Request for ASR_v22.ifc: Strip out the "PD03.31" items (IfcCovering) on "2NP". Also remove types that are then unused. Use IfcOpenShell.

First a look at what the model holds.

```python
import ifcopenshell
import ifcopenshell.util.element

model = ifcopenshell.open("ASR_v22.ifc")
print(model.schema)
storey = next(s for s in model.by_type("IfcBuildingStorey") if s.Name == "2NP")
coverings = [e for e in ifcopenshell.util.element.get_decomposition(storey) if e.is_a("IfcCovering")]
seen = {}
for e in coverings:
    element_type = ifcopenshell.util.element.get_type(e)
    name = element_type.Name if element_type not in (None, e) else None
    seen[name] = seen.get(name, 0) + 1
for name, count in sorted(seen.items(), key=str):
    print(count, "x", name)
```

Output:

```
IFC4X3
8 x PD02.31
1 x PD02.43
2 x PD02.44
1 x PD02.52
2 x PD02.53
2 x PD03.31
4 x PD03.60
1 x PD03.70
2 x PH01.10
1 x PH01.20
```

```python
import ifcopenshell
import ifcopenshell.api.root
import ifcopenshell.util.element

model = ifcopenshell.open("ASR_v22.ifc")

storey = next(s for s in model.by_type("IfcBuildingStorey") if s.Name == "2NP")
coverings = [e for e in ifcopenshell.util.element.get_decomposition(storey) if e.is_a("IfcCovering")]
targets = [e for e in coverings if (t := ifcopenshell.util.element.get_type(e)) not in (None, e) and t.Name == "PD03.31"]
types = {ifcopenshell.util.element.get_type(e) for e in targets} - {None, *targets}

for e in targets:
    ifcopenshell.api.root.remove_product(model, product=e)
print(len(targets), "removed")

unused = [t for t in types if not ifcopenshell.util.element.get_types(t)]
for t in unused:
    ifcopenshell.api.root.remove_product(model, product=t)
print(len(unused), "unused types removed")

model.write("ASR_v22_updated.ifc")
```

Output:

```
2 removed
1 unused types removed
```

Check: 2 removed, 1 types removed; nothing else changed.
